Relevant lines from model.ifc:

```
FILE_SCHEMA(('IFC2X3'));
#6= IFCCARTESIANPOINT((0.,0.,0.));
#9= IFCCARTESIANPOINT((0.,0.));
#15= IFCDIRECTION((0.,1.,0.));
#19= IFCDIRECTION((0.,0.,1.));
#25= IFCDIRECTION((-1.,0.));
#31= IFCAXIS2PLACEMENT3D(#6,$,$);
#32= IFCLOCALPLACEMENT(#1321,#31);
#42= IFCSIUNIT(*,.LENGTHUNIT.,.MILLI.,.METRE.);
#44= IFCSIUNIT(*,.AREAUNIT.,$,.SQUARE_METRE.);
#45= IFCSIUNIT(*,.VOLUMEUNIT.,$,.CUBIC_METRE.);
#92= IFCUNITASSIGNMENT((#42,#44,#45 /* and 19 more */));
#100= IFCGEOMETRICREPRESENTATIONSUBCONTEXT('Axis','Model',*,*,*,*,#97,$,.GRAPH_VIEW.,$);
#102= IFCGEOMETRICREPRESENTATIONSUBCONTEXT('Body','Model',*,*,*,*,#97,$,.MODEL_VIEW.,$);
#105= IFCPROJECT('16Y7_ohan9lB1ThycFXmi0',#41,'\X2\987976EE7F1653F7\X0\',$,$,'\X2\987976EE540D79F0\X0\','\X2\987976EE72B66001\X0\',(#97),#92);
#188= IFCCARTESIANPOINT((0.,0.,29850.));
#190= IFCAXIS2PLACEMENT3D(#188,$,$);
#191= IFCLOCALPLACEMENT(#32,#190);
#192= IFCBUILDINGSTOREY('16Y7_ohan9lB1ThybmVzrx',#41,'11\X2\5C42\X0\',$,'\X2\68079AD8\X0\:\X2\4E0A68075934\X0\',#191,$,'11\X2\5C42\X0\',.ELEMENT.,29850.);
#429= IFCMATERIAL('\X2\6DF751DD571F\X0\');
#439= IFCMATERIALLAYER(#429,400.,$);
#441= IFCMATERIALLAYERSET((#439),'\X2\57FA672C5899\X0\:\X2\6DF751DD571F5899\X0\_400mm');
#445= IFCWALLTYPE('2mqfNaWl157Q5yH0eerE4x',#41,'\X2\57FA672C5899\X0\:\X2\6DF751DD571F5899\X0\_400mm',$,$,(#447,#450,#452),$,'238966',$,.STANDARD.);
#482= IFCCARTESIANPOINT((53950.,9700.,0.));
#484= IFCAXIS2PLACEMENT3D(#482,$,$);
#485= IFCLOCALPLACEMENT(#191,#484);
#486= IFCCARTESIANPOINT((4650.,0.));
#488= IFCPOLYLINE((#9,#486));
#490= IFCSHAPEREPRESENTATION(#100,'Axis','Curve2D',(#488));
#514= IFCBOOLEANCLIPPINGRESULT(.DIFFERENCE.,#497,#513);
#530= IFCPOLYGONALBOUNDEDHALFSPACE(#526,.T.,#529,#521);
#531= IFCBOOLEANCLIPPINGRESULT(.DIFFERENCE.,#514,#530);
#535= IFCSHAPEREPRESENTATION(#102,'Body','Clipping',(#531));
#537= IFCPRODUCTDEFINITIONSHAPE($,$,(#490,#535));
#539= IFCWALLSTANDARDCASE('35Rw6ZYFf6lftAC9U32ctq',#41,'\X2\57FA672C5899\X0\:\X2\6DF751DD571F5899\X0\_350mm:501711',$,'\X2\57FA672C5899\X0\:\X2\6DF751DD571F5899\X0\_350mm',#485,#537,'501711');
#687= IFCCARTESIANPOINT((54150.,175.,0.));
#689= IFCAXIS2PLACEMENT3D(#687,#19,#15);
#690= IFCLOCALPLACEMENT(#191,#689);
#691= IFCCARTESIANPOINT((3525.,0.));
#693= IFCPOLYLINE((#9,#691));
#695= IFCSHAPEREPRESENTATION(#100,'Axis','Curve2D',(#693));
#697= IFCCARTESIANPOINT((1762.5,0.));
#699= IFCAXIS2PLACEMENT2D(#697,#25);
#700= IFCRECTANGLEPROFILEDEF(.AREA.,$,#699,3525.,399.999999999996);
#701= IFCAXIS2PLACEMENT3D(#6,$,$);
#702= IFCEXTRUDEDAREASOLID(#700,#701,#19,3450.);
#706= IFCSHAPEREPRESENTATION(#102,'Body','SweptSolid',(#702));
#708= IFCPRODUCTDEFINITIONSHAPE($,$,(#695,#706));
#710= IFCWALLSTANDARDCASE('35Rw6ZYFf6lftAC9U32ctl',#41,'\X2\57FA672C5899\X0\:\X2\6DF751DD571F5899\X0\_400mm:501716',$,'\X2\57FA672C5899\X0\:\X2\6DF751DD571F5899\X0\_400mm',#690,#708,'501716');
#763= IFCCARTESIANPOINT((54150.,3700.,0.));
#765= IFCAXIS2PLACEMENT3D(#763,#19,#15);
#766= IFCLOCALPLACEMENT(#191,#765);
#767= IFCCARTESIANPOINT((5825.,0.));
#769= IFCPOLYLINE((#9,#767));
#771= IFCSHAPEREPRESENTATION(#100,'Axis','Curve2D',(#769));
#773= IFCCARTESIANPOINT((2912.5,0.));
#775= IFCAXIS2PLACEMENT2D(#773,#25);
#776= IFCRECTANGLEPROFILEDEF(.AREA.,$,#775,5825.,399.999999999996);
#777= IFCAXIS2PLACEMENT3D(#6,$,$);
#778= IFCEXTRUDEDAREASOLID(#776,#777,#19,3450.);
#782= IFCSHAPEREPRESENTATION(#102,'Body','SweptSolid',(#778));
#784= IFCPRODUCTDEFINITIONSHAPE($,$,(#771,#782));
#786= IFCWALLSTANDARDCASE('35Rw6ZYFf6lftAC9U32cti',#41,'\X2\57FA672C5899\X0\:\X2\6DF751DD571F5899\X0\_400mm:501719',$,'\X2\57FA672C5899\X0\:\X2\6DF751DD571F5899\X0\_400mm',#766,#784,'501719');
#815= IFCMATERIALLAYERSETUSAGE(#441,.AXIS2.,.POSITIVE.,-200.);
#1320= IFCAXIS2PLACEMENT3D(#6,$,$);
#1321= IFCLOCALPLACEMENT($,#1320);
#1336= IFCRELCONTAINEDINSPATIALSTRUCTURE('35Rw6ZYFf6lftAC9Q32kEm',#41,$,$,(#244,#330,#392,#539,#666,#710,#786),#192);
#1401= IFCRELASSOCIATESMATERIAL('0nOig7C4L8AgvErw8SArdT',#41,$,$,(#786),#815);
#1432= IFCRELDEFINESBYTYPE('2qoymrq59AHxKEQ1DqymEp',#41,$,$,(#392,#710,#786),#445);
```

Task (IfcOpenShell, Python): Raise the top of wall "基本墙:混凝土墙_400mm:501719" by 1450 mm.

```python
import ifcopenshell
import ifcopenshell.geom
import ifcopenshell.util.representation
import ifcopenshell.util.shape
import ifcopenshell.util.unit

model = ifcopenshell.open("model.ifc")
unit_scale = ifcopenshell.util.unit.calculate_unit_scale(model)
settings = ifcopenshell.geom.settings()


def volume(element):
    """Net volume in cubic metres, openings subtracted."""
    shape = ifcopenshell.geom.create_shape(settings, element)
    return ifcopenshell.util.shape.get_volume(shape.geometry)


wall = model.by_guid("35Rw6ZYFf6lftAC9U32cti")
before = volume(wall)

body = ifcopenshell.util.representation.get_representation(wall, "Model", "Body")
solid = body.Items[0]
old_height = solid.Depth
solid.Depth += 1.45 / unit_scale
after = volume(wall)

print(f"height {old_height:g} -> {solid.Depth:g}, volume {before:.3f} -> {after:.3f} m3")

model.write("model_v2.ifc")
```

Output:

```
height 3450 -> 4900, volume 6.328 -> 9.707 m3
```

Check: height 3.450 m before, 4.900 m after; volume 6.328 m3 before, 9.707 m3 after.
